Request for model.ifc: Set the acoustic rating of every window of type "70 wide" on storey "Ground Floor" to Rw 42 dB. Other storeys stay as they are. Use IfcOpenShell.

First a look at what the model holds.

```python
import ifcopenshell
import ifcopenshell.util.element

model = ifcopenshell.open("model.ifc")
print(model.schema)
storey = next(s for s in model.by_type("IfcBuildingStorey") if s.Name == "Ground Floor")
windows = [e for e in ifcopenshell.util.element.get_decomposition(storey) if e.is_a("IfcWindow")]
seen = {}
for e in windows:
    element_type = ifcopenshell.util.element.get_type(e)
    key = (element_type.Name if element_type != e and element_type else None, ifcopenshell.util.element.get_pset(e, "Pset_WindowCommon", "AcousticRating"))
    seen[key] = seen.get(key, 0) + 1
for (name, value), count in sorted(seen.items(), key=str):
    print(count, "x", name, "|", value)
```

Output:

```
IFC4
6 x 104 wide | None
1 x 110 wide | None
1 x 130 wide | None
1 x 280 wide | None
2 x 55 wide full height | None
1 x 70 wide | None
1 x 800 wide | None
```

```python
import ifcopenshell
import ifcopenshell.api.pset
import ifcopenshell.util.element

model = ifcopenshell.open("model.ifc")

storey = next(s for s in model.by_type("IfcBuildingStorey") if s.Name == "Ground Floor")
windows = [e for e in ifcopenshell.util.element.get_decomposition(storey) if e.is_a("IfcWindow")]

count = 0
for e in windows:
    element_type = ifcopenshell.util.element.get_type(e)
    if element_type in (None, e) or element_type.Name != "70 wide":
        continue
    # add_pset returns the element's existing set when there is one.
    pset = ifcopenshell.api.pset.add_pset(model, product=e, name="Pset_WindowCommon")
    ifcopenshell.api.pset.edit_pset(model, pset=pset, properties={"AcousticRating": "Rw 42 dB"})
    count += 1

print(count, "windows updated")

model.write("model-out.ifc")
```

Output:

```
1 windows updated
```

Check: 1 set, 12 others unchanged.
